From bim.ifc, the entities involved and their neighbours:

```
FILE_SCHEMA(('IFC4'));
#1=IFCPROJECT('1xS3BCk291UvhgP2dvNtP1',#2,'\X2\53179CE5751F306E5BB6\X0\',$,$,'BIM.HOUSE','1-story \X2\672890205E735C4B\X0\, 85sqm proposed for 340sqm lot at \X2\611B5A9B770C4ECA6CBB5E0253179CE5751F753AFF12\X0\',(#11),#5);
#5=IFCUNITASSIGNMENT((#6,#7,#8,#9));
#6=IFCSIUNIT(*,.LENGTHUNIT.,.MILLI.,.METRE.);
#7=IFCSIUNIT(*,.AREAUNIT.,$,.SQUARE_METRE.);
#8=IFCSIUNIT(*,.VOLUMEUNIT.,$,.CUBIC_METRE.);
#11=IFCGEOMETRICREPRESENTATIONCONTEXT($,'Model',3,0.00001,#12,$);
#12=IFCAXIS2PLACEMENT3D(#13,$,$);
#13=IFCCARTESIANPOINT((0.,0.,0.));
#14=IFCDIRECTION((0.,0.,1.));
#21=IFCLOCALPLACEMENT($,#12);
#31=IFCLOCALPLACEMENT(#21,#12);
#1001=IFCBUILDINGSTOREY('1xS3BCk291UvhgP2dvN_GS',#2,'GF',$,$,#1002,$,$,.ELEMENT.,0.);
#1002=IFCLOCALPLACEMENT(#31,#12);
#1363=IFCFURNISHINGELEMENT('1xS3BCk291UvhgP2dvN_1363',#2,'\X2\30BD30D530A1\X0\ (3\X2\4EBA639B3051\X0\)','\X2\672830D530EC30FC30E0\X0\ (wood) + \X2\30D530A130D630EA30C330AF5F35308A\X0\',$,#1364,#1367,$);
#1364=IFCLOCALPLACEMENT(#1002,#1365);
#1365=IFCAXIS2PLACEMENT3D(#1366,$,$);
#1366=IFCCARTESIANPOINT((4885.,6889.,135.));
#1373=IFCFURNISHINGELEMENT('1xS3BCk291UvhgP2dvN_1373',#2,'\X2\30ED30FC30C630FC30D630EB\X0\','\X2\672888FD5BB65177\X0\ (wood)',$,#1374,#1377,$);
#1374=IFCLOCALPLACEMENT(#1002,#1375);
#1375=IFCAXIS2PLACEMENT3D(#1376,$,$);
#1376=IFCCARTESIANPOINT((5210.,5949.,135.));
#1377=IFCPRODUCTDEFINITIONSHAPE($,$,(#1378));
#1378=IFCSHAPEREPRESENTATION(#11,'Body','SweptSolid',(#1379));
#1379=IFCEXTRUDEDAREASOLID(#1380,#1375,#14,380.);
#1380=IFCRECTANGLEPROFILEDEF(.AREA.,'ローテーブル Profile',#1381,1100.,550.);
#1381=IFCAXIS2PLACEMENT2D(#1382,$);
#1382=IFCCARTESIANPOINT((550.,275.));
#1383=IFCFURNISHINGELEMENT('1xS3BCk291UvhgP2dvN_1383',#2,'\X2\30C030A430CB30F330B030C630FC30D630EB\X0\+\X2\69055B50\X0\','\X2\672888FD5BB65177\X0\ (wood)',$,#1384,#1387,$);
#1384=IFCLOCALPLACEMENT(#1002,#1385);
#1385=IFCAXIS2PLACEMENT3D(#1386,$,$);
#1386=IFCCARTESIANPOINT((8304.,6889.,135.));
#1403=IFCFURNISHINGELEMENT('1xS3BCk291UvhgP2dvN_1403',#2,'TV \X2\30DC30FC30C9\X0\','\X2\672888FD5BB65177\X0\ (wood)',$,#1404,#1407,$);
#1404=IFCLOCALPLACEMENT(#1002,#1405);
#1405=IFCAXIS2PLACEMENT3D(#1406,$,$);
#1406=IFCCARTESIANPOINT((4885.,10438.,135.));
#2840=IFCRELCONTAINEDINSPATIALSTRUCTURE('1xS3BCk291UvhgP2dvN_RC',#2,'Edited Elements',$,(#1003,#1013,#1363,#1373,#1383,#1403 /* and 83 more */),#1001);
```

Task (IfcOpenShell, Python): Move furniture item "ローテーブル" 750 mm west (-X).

```python
import ifcopenshell
import ifcopenshell.api.geometry
import ifcopenshell.util.placement
import ifcopenshell.util.unit

model = ifcopenshell.open("bim.ifc")
unit_scale = ifcopenshell.util.unit.calculate_unit_scale(model)

item = model.by_id(1373)
matrix = ifcopenshell.util.placement.get_local_placement(item.ObjectPlacement)
matrix[0, 3] -= 0.75 / unit_scale
ifcopenshell.api.geometry.edit_object_placement(model, product=item, matrix=matrix, is_si=False)

print(ifcopenshell.util.placement.get_local_placement(item.ObjectPlacement).round(3) + 0.0)

model.write("bim_updated.ifc")
```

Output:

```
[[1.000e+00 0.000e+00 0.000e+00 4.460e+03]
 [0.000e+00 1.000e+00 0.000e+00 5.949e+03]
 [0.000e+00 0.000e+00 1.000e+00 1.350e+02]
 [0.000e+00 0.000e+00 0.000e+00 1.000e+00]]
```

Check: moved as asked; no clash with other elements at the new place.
